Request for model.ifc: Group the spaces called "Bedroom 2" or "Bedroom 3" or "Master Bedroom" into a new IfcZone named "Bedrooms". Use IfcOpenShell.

First a look at what the model holds.

```python
import ifcopenshell

model = ifcopenshell.open("model.ifc")
print(model.schema)
seen = {}
for space in model.by_type("IfcSpace"):
    seen[space.LongName] = seen.get(space.LongName, 0) + 1
for name, count in sorted(seen.items(), key=str):
    print(count, "x", name)
print("zones:", [z.Name for z in model.by_type("IfcZone")][:20])
```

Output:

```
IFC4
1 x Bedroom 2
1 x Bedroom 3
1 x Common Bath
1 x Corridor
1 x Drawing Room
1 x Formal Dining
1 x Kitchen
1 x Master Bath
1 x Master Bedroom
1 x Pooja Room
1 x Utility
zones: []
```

```python
import ifcopenshell
import ifcopenshell.api.group
import ifcopenshell.api.root

model = ifcopenshell.open("model.ifc")

names = {"Bedroom 2", "Bedroom 3", "Master Bedroom"}
spaces = [s for s in model.by_type("IfcSpace") if s.LongName in names]

zone = ifcopenshell.api.root.create_entity(model, ifc_class="IfcZone", name="Bedrooms")
ifcopenshell.api.group.assign_group(model, products=spaces, group=zone)
print(len(spaces), "spaces in", zone.Name)

model.write("model-out.ifc")
```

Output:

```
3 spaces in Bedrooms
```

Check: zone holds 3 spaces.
